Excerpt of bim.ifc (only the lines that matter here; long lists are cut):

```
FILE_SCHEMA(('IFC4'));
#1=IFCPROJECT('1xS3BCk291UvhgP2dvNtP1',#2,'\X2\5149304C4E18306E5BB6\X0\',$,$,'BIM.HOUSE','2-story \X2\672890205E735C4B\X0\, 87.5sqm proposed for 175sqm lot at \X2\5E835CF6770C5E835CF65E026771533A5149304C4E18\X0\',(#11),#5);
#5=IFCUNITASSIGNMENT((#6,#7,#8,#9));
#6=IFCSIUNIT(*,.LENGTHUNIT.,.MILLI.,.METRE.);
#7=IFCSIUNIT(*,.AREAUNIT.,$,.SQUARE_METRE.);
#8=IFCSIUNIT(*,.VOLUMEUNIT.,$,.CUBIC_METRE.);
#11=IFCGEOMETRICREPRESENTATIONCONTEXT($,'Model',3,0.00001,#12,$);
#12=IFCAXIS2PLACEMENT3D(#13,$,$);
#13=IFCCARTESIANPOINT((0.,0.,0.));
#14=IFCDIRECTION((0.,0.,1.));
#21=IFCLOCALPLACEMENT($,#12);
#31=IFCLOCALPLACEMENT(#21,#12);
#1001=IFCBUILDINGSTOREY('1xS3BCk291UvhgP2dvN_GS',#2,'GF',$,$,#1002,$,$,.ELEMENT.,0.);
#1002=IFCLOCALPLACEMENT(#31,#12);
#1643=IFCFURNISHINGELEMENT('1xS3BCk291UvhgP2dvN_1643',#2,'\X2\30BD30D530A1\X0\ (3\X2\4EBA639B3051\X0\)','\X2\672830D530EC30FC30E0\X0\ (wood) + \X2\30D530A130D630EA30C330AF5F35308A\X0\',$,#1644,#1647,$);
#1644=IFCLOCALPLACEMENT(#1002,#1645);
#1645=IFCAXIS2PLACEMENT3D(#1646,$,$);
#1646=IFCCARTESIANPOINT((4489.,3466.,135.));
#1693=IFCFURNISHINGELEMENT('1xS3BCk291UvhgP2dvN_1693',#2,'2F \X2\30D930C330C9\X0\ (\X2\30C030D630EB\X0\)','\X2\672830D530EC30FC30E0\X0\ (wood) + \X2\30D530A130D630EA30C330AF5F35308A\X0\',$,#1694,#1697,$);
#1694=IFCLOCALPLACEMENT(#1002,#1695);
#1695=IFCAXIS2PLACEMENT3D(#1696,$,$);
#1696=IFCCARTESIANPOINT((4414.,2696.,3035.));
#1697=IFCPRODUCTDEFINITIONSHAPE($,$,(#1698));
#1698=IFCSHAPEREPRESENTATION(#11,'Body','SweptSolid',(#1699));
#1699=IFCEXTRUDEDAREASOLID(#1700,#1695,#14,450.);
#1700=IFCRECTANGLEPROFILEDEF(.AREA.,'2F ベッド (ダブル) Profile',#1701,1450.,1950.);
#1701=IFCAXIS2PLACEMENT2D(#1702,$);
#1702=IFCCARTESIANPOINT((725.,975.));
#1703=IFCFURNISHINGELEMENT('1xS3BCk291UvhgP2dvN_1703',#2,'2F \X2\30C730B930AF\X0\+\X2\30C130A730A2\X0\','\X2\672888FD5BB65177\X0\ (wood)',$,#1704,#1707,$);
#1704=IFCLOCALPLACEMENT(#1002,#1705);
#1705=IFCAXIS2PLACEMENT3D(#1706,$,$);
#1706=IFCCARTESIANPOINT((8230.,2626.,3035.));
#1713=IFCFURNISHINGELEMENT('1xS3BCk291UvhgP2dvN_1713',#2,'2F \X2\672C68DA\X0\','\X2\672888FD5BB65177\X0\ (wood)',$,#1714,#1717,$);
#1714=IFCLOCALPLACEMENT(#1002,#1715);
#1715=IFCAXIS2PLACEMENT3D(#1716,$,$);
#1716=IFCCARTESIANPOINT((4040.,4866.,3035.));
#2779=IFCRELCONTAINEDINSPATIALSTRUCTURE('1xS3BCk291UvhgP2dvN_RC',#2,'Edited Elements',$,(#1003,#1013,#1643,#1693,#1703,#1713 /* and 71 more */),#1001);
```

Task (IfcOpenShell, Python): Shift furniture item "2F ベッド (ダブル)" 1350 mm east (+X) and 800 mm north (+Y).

```python
import ifcopenshell
import ifcopenshell.api.geometry
import ifcopenshell.util.placement
import ifcopenshell.util.unit

model = ifcopenshell.open("bim.ifc")
unit_scale = ifcopenshell.util.unit.calculate_unit_scale(model)

item = model.by_guid("1xS3BCk291UvhgP2dvN_1693")
matrix = ifcopenshell.util.placement.get_local_placement(item.ObjectPlacement)
matrix[0, 3] += 1.35 / unit_scale
matrix[1, 3] += 0.8 / unit_scale
ifcopenshell.api.geometry.edit_object_placement(model, product=item, matrix=matrix, is_si=False)

print(ifcopenshell.util.placement.get_local_placement(item.ObjectPlacement).round(3) + 0.0)

model.write("bim_v2.ifc")
```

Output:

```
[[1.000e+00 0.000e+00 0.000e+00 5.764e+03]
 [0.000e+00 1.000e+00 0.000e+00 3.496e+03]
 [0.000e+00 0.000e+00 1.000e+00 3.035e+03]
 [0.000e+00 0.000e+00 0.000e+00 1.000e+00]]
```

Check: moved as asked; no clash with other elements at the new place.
